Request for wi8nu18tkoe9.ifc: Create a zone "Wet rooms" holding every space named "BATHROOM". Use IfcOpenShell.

First a look at what the model holds.

```python
import ifcopenshell

model = ifcopenshell.open("wi8nu18tkoe9.ifc")
print(model.schema)
seen = {}
for space in model.by_type("IfcSpace"):
    seen[space.LongName] = seen.get(space.LongName, 0) + 1
for name, count in sorted(seen.items(), key=str):
    print(count, "x", name)
print("zones:", [z.Name for z in model.by_type("IfcZone")][:20])
```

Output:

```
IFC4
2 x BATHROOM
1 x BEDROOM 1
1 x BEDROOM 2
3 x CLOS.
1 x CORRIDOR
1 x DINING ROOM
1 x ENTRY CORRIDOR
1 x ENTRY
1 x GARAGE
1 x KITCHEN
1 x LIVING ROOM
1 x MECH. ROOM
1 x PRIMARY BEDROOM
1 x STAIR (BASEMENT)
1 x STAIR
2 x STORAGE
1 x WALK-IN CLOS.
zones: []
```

```python
import ifcopenshell
import ifcopenshell.api.group
import ifcopenshell.api.root

model = ifcopenshell.open("wi8nu18tkoe9.ifc")

names = {"BATHROOM"}
spaces = [s for s in model.by_type("IfcSpace") if s.LongName in names]

zone = ifcopenshell.api.root.create_entity(model, ifc_class="IfcZone", name="Wet rooms")
ifcopenshell.api.group.assign_group(model, products=spaces, group=zone)
print(len(spaces), "spaces in", zone.Name)

model.write("wi8nu18tkoe9_edited.ifc")
```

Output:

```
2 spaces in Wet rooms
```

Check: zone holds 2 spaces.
